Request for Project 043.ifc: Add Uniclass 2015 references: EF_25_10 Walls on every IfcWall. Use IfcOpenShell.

First a look at what the model holds.

```python
import ifcopenshell

model = ifcopenshell.open("Project 043.ifc")
print(model.schema)
print("classifications:", [c.Name for c in model.by_type("IfcClassification")])
for ifc_class in ("IfcDoor", "IfcRoof", "IfcStair", "IfcWall", "IfcWindow"):
    print(ifc_class, len(model.by_type(ifc_class)))
```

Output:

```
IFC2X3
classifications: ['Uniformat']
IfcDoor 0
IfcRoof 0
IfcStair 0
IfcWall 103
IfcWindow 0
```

```python
import ifcopenshell
import ifcopenshell.api.classification

model = ifcopenshell.open("Project 043.ifc")

# IFC2X3 requires Source and Edition and has no link from the project to the system.
system = model.create_entity("IfcClassification", Source="NBS", Edition="2015", Name="Uniclass 2015")

codes = {
    "IfcWall": ("EF_25_10", "Walls"),
}
for ifc_class, (code, name) in codes.items():
    products = model.by_type(ifc_class)
    ifcopenshell.api.classification.add_reference(
        model, products=products, classification=system, identification=code, name=name
    )
    print(code, len(products))

model.write("Project 043-out.ifc")
```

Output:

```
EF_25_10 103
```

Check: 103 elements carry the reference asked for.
